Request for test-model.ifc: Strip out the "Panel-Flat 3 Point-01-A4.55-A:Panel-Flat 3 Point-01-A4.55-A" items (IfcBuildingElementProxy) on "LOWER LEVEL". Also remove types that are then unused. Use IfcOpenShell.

First a look at what the model holds.

```python
import ifcopenshell
import ifcopenshell.util.element

model = ifcopenshell.open("test-model.ifc")
print(model.schema)
storey = next(s for s in model.by_type("IfcBuildingStorey") if s.Name == "LOWER LEVEL")
proxies = [e for e in ifcopenshell.util.element.get_decomposition(storey) if e.is_a("IfcBuildingElementProxy")]
seen = {}
for e in proxies:
    element_type = ifcopenshell.util.element.get_type(e)
    name = element_type.Name if element_type not in (None, e) else None
    seen[name] = seen.get(name, 0) + 1
for name, count in sorted(seen.items(), key=str):
    print(count, "x", name)
```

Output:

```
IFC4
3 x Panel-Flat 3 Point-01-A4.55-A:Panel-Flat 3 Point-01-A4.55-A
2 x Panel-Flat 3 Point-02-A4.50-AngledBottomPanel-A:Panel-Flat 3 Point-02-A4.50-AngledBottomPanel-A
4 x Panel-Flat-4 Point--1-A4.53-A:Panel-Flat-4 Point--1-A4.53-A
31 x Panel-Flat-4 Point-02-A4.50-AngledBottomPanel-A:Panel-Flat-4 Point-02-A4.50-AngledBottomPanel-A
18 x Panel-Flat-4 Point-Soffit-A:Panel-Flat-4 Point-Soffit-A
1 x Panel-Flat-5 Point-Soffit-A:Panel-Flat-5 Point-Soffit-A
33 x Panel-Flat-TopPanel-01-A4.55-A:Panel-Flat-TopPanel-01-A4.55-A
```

```python
import ifcopenshell
import ifcopenshell.api.root
import ifcopenshell.util.element

model = ifcopenshell.open("test-model.ifc")

storey = next(s for s in model.by_type("IfcBuildingStorey") if s.Name == "LOWER LEVEL")
proxies = [e for e in ifcopenshell.util.element.get_decomposition(storey) if e.is_a("IfcBuildingElementProxy")]
targets = [e for e in proxies if (t := ifcopenshell.util.element.get_type(e)) not in (None, e) and t.Name == "Panel-Flat 3 Point-01-A4.55-A:Panel-Flat 3 Point-01-A4.55-A"]
types = {ifcopenshell.util.element.get_type(e) for e in targets} - {None, *targets}

for e in targets:
    ifcopenshell.api.root.remove_product(model, product=e)
print(len(targets), "removed")

unused = [t for t in types if not ifcopenshell.util.element.get_types(t)]
for t in unused:
    ifcopenshell.api.root.remove_product(model, product=t)
print(len(unused), "unused types removed")

model.write("test-model_updated.ifc")
```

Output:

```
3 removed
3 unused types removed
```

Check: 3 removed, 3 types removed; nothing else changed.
